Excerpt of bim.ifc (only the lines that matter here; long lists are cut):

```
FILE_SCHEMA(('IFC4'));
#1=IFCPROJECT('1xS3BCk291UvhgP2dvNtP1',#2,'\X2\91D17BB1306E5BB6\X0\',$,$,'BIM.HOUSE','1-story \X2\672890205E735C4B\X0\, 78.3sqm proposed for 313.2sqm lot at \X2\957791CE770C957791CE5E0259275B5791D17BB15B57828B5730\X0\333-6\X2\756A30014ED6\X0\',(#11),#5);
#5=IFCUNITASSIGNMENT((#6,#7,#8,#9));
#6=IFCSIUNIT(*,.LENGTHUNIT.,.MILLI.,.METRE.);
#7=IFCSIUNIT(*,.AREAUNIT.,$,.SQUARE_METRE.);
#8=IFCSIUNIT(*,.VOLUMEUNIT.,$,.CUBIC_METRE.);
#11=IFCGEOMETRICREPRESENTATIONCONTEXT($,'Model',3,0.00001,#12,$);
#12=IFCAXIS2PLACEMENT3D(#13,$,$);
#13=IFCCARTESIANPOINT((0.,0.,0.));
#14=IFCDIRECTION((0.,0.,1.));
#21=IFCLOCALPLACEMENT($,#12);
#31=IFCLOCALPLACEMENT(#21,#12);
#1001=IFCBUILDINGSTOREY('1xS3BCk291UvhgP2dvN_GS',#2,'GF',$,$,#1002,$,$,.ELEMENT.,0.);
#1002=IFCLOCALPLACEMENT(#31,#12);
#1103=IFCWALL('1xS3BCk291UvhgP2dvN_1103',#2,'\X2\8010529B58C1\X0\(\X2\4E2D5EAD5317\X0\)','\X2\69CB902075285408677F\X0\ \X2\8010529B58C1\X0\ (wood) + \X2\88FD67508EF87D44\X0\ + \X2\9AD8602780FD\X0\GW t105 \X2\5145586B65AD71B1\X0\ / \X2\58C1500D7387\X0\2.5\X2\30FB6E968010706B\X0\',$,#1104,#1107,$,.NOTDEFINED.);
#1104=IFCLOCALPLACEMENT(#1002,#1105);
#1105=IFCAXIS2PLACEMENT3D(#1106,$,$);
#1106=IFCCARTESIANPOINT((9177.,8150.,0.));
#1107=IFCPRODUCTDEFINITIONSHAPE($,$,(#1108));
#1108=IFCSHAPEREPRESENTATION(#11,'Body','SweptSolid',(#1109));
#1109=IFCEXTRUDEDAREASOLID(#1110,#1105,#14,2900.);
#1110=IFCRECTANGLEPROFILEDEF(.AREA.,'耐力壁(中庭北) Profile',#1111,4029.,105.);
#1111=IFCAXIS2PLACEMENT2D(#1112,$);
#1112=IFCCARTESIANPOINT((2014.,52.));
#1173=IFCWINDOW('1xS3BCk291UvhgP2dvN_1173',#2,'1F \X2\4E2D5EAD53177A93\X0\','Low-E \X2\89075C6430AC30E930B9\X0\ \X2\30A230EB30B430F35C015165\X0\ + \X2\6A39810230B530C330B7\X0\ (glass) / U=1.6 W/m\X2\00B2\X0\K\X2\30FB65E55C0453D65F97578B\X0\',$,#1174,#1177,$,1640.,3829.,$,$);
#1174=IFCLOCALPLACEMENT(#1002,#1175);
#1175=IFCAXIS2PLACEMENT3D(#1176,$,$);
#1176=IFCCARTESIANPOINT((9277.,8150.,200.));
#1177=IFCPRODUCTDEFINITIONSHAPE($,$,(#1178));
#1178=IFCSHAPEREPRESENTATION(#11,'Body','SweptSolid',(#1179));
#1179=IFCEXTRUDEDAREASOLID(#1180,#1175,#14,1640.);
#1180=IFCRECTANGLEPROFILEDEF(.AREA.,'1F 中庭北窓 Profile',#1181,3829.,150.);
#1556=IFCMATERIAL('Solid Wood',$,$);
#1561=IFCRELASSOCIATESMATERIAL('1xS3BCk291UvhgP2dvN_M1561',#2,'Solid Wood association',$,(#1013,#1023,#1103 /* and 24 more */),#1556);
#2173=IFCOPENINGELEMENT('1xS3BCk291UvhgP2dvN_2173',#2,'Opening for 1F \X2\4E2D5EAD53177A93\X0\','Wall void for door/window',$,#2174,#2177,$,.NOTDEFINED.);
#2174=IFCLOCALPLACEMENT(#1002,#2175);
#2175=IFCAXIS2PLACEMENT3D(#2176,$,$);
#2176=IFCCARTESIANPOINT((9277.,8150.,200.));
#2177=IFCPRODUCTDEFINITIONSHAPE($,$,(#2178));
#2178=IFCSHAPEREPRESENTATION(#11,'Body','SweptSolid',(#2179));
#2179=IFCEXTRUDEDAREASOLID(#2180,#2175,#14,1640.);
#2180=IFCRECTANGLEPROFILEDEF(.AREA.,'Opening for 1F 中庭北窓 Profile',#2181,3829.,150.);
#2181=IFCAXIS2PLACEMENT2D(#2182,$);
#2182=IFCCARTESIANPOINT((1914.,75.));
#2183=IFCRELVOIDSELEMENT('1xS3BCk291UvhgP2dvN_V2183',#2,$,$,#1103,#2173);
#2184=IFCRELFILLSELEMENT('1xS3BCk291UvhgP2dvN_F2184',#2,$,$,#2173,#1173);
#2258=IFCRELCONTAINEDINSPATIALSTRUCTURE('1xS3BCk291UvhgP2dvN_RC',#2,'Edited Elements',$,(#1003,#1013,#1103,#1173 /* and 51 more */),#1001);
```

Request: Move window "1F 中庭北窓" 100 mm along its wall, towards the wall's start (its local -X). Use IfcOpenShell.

```python
import ifcopenshell
import ifcopenshell.api.geometry
import ifcopenshell.util.placement
import ifcopenshell.util.unit

model = ifcopenshell.open("bim.ifc")
unit_scale = ifcopenshell.util.unit.calculate_unit_scale(model)

window = model.by_guid("1xS3BCk291UvhgP2dvN_1173")
opening = window.FillsVoids[0].RelatingOpeningElement
wall = opening.VoidsElements[0].RelatingBuildingElement

wall_matrix = ifcopenshell.util.placement.get_local_placement(wall.ObjectPlacement)
shift = wall_matrix[:3, 0] * -0.1 / unit_scale
before = ifcopenshell.util.placement.get_local_placement(window.ObjectPlacement)[:3, 3].copy()

# The window is not placed relative to its opening, so move both.
for product in (opening, window):
    matrix = ifcopenshell.util.placement.get_local_placement(product.ObjectPlacement)
    matrix[:3, 3] += shift
    ifcopenshell.api.geometry.edit_object_placement(model, product=product, matrix=matrix, is_si=False)

after = ifcopenshell.util.placement.get_local_placement(window.ObjectPlacement)[:3, 3]
print("window moved by", (after - before).round(3) + 0.0)

model.write("bim_v2.ifc")
```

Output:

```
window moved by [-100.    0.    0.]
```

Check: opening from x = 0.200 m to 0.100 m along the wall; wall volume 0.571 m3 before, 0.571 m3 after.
